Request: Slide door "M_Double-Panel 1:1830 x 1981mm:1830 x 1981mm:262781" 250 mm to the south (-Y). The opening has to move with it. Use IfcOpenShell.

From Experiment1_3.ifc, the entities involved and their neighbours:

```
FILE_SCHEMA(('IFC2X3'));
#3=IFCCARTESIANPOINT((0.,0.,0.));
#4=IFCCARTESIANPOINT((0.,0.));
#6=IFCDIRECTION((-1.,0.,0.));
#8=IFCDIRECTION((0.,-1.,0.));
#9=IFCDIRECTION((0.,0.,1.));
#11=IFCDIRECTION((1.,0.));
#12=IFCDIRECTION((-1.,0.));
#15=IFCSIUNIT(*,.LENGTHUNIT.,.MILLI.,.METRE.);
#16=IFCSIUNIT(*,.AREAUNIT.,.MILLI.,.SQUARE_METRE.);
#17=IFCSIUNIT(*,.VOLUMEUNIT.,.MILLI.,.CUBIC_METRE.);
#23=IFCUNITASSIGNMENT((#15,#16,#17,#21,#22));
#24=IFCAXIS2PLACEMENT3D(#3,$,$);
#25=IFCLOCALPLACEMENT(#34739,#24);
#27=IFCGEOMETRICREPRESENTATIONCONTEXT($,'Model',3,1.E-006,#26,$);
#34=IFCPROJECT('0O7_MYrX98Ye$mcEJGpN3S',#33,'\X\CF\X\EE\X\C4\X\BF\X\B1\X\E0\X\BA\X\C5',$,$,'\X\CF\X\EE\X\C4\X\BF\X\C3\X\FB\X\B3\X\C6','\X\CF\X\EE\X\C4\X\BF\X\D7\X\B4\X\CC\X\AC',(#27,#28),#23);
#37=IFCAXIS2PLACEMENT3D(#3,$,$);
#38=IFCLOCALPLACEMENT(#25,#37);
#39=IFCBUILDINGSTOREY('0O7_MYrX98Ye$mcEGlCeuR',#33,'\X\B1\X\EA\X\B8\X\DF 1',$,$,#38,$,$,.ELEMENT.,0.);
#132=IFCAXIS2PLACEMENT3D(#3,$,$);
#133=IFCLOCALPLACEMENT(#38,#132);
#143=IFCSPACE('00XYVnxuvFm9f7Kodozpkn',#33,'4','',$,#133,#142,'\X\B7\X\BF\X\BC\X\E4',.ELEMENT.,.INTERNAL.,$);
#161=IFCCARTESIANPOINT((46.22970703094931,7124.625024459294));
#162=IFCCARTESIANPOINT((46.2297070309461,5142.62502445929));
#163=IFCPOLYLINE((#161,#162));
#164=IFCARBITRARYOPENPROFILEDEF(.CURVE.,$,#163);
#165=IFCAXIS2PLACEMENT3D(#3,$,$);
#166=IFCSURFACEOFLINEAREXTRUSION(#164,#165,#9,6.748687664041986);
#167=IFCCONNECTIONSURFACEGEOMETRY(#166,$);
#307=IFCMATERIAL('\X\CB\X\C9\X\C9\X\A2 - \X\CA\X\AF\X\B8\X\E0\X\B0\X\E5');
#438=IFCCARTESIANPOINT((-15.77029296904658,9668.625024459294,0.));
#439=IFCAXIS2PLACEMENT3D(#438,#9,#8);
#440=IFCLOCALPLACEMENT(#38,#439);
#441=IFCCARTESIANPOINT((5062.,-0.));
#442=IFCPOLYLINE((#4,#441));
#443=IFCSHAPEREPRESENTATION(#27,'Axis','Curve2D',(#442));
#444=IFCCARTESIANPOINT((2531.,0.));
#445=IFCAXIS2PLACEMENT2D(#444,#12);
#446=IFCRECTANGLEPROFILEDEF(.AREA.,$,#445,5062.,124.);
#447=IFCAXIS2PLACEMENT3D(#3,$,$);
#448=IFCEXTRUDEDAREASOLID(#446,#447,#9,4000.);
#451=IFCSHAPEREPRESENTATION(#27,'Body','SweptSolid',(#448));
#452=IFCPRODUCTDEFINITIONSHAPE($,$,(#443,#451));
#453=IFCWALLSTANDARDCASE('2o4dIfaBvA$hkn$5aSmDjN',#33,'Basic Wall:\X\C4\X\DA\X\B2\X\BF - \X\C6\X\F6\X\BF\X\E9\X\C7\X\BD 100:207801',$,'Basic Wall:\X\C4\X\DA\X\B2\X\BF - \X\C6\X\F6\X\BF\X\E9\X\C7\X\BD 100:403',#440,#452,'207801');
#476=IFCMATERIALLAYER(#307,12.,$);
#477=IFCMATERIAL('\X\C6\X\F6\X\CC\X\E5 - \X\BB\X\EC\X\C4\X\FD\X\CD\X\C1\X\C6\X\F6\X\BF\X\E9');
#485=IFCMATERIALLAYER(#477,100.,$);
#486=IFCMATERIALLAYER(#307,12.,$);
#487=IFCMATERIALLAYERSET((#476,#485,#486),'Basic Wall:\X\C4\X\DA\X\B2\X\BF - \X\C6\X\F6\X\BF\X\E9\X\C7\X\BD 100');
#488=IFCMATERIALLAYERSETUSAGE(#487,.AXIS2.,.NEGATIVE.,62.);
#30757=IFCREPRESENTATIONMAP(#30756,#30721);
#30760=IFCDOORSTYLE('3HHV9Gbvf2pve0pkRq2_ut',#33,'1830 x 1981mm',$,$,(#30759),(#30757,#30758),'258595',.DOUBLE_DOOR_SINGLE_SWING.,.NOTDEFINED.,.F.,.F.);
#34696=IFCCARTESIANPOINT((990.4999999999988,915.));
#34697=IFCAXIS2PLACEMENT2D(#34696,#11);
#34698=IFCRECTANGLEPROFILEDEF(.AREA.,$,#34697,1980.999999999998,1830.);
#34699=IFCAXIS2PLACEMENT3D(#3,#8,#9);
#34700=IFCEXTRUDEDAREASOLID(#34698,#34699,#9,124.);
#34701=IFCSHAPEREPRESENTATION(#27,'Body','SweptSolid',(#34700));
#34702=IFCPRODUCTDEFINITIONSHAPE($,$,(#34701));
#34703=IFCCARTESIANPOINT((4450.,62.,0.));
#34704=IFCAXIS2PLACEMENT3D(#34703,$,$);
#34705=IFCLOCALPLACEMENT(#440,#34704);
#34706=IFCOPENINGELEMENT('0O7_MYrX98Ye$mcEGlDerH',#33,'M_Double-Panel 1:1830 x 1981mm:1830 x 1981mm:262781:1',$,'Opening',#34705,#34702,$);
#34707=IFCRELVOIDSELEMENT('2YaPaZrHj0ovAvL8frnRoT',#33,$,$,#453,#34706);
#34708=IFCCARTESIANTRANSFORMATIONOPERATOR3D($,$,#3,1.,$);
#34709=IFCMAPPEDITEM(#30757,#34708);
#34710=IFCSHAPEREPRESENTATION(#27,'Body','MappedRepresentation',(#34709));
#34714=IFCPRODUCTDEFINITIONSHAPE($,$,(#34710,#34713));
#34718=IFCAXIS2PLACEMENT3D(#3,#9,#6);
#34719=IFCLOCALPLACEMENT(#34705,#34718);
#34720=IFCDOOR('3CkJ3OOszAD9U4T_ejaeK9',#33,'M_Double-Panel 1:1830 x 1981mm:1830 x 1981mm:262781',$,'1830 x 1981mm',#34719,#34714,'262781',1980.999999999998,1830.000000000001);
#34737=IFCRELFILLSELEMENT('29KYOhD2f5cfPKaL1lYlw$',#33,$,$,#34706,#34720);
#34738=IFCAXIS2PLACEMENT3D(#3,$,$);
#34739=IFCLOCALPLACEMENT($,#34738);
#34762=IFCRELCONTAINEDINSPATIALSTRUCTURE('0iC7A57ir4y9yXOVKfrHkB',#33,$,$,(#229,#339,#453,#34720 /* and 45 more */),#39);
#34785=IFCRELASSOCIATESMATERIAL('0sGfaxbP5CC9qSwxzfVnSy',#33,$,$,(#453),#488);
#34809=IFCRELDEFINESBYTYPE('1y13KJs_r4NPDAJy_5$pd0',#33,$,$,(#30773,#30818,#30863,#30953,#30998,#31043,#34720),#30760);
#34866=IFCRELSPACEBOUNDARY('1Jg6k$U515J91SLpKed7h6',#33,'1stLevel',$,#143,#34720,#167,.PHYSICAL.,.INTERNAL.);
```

```python
import numpy as np
import ifcopenshell
import ifcopenshell.api.geometry
import ifcopenshell.util.placement

model = ifcopenshell.open("Experiment1_3.ifc")

door = model.by_id(34720)
opening = door.FillsVoids[0].RelatingOpeningElement
wall = opening.VoidsElements[0].RelatingBuildingElement

wall_matrix = ifcopenshell.util.placement.get_local_placement(wall.ObjectPlacement)
shift = wall_matrix[:3, 0] * 250.0
before = ifcopenshell.util.placement.get_local_placement(door.ObjectPlacement)[:3, 3].copy()

# The door is placed relative to its opening, so it follows when the opening moves.
matrix = ifcopenshell.util.placement.get_local_placement(opening.ObjectPlacement)
matrix[:3, 3] += shift
ifcopenshell.api.geometry.edit_object_placement(
    model, product=opening, matrix=matrix, is_si=False, should_transform_children=True
)

# Space boundary surfaces are stored in each space's coordinates; move them too.
for rel in door.ProvidesBoundaries:
    if not rel.ConnectionGeometry:
        continue
    surface = rel.ConnectionGeometry.SurfaceOnRelatingElement
    space_matrix = ifcopenshell.util.placement.get_local_placement(rel.RelatingSpace.ObjectPlacement)
    point = np.array(surface.Position.Location.Coordinates) + space_matrix[:3, :3].T @ shift
    surface.Position = model.createIfcAxis2Placement3D(
        model.createIfcCartesianPoint(point.tolist()), surface.Position.Axis, surface.Position.RefDirection
    )

after = ifcopenshell.util.placement.get_local_placement(door.ObjectPlacement)[:3, 3]
print("door moved by", (after - before).round(3) + 0.0)

model.write("Experiment1_3_v2.ifc")
```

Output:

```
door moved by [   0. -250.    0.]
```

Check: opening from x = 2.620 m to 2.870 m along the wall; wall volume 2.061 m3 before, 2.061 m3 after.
